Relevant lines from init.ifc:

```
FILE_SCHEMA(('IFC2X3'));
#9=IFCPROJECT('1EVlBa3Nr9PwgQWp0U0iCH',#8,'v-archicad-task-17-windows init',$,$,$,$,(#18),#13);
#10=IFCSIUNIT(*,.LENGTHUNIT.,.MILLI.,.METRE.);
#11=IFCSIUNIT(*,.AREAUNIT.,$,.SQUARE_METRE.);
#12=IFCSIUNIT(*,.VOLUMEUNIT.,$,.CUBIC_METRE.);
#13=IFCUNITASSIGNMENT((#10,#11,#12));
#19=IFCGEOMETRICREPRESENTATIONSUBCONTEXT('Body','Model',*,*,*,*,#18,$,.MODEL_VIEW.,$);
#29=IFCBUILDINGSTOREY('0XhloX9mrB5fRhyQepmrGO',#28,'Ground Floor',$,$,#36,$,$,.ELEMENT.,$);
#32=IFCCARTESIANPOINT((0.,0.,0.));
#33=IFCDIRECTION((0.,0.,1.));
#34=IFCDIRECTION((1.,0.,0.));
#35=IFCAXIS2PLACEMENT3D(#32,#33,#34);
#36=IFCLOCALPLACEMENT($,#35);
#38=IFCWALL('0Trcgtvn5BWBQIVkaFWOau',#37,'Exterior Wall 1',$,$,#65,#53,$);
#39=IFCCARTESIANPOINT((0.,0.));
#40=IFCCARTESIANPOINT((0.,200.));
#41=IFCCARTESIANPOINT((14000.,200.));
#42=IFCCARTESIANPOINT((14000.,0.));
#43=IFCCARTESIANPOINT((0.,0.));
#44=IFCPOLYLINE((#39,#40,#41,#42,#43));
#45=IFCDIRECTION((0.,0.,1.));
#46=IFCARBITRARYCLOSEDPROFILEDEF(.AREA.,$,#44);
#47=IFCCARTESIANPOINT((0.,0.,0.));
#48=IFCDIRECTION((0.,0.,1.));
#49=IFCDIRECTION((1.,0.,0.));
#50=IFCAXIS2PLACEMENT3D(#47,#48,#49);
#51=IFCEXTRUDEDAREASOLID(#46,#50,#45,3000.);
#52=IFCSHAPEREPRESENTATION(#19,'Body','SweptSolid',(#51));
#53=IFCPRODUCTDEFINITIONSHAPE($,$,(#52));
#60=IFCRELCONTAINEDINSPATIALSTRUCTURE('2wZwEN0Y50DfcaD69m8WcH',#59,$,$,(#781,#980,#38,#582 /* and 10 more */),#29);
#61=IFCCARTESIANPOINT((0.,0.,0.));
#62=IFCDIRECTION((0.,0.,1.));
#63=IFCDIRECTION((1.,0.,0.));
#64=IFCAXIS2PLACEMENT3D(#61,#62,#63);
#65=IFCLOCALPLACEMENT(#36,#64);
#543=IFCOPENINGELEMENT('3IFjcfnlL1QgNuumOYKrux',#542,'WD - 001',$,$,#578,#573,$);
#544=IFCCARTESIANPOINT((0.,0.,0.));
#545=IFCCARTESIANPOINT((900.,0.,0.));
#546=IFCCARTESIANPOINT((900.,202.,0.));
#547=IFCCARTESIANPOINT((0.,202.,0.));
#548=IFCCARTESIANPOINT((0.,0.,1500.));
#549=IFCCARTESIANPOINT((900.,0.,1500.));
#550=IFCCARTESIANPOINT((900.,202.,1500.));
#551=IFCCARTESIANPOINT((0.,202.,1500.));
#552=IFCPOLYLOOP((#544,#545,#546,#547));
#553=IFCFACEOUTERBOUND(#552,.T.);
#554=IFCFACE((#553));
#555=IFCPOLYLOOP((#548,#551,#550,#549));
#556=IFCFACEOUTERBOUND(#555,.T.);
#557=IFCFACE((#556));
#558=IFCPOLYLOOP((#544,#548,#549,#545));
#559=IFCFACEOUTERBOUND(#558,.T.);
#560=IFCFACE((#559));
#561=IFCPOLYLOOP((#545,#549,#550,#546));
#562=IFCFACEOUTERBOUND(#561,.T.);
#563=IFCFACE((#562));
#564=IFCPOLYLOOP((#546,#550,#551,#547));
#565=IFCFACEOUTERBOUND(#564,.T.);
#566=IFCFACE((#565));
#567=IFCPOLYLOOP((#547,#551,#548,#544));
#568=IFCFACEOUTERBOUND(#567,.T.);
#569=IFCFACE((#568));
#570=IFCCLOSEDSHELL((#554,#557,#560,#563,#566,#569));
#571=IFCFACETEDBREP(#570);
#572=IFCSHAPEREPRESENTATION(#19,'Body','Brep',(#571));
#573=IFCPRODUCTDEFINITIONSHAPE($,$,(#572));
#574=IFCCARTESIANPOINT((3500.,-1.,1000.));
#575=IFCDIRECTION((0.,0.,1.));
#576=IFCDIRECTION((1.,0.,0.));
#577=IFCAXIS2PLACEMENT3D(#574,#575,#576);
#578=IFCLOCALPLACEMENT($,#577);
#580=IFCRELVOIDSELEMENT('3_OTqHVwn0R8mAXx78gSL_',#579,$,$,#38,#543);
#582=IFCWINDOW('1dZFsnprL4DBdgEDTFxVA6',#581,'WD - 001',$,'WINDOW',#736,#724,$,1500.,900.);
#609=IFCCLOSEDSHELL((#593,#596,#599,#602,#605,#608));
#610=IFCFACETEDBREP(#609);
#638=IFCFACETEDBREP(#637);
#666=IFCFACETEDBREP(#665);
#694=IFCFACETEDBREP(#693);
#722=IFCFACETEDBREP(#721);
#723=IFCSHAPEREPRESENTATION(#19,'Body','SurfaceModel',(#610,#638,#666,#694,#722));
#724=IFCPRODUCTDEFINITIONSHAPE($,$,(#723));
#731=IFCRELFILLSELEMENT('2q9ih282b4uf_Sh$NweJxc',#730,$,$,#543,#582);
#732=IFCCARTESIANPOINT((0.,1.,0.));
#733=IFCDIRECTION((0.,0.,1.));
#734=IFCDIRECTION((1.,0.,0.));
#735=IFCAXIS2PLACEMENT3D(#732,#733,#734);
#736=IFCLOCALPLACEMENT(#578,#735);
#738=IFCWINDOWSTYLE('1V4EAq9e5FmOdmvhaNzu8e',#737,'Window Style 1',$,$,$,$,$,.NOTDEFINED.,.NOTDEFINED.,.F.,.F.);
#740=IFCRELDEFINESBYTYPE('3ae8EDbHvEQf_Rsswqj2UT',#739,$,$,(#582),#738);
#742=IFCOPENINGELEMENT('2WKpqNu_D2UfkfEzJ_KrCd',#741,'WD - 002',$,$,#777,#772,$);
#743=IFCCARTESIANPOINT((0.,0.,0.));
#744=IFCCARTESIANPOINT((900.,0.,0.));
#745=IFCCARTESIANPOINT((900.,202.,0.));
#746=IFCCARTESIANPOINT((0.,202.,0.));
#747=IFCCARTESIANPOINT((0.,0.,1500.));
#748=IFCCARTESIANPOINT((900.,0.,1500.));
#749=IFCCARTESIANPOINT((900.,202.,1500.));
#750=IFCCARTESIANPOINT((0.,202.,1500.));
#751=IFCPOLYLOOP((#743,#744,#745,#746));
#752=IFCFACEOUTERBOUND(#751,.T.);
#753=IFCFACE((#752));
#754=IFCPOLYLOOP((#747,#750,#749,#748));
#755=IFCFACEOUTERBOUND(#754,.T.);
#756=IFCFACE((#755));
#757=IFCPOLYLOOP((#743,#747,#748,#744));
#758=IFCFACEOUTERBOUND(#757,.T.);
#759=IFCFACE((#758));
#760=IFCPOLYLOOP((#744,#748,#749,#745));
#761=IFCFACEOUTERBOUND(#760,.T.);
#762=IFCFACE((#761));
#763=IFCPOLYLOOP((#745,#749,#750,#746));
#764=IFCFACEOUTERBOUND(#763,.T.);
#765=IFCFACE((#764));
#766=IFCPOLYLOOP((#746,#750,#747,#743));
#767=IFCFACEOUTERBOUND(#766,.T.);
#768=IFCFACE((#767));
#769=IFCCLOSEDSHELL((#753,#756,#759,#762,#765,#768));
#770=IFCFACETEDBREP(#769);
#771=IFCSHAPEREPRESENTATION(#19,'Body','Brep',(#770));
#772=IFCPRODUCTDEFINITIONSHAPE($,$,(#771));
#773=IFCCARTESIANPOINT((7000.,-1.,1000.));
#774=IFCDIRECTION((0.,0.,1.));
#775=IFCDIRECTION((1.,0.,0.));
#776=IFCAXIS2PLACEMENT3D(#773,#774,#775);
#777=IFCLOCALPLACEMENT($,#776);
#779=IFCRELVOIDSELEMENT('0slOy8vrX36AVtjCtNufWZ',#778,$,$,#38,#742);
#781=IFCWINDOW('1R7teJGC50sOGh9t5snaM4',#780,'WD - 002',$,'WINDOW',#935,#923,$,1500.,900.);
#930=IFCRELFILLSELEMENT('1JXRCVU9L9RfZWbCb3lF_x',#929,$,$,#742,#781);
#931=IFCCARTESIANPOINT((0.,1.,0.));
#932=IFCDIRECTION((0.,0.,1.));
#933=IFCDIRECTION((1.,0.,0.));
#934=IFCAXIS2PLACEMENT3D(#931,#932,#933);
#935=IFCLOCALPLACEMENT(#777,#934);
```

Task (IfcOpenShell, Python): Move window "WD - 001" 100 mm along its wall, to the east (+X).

```python
import ifcopenshell
import ifcopenshell.api.geometry
import ifcopenshell.util.placement

model = ifcopenshell.open("init.ifc")

window = model.by_guid("1dZFsnprL4DBdgEDTFxVA6")
opening = window.FillsVoids[0].RelatingOpeningElement
wall = opening.VoidsElements[0].RelatingBuildingElement

wall_matrix = ifcopenshell.util.placement.get_local_placement(wall.ObjectPlacement)
shift = wall_matrix[:3, 0] * 100.0
before = ifcopenshell.util.placement.get_local_placement(window.ObjectPlacement)[:3, 3].copy()

# The window is placed relative to its opening, so it follows when the opening moves.
matrix = ifcopenshell.util.placement.get_local_placement(opening.ObjectPlacement)
matrix[:3, 3] += shift
ifcopenshell.api.geometry.edit_object_placement(
    model, product=opening, matrix=matrix, is_si=False, should_transform_children=True
)

after = ifcopenshell.util.placement.get_local_placement(window.ObjectPlacement)[:3, 3]
print("window moved by", (after - before).round(3) + 0.0)

model.write("init_v2.ifc")
```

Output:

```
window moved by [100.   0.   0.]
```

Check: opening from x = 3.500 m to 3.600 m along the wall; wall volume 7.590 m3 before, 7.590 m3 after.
